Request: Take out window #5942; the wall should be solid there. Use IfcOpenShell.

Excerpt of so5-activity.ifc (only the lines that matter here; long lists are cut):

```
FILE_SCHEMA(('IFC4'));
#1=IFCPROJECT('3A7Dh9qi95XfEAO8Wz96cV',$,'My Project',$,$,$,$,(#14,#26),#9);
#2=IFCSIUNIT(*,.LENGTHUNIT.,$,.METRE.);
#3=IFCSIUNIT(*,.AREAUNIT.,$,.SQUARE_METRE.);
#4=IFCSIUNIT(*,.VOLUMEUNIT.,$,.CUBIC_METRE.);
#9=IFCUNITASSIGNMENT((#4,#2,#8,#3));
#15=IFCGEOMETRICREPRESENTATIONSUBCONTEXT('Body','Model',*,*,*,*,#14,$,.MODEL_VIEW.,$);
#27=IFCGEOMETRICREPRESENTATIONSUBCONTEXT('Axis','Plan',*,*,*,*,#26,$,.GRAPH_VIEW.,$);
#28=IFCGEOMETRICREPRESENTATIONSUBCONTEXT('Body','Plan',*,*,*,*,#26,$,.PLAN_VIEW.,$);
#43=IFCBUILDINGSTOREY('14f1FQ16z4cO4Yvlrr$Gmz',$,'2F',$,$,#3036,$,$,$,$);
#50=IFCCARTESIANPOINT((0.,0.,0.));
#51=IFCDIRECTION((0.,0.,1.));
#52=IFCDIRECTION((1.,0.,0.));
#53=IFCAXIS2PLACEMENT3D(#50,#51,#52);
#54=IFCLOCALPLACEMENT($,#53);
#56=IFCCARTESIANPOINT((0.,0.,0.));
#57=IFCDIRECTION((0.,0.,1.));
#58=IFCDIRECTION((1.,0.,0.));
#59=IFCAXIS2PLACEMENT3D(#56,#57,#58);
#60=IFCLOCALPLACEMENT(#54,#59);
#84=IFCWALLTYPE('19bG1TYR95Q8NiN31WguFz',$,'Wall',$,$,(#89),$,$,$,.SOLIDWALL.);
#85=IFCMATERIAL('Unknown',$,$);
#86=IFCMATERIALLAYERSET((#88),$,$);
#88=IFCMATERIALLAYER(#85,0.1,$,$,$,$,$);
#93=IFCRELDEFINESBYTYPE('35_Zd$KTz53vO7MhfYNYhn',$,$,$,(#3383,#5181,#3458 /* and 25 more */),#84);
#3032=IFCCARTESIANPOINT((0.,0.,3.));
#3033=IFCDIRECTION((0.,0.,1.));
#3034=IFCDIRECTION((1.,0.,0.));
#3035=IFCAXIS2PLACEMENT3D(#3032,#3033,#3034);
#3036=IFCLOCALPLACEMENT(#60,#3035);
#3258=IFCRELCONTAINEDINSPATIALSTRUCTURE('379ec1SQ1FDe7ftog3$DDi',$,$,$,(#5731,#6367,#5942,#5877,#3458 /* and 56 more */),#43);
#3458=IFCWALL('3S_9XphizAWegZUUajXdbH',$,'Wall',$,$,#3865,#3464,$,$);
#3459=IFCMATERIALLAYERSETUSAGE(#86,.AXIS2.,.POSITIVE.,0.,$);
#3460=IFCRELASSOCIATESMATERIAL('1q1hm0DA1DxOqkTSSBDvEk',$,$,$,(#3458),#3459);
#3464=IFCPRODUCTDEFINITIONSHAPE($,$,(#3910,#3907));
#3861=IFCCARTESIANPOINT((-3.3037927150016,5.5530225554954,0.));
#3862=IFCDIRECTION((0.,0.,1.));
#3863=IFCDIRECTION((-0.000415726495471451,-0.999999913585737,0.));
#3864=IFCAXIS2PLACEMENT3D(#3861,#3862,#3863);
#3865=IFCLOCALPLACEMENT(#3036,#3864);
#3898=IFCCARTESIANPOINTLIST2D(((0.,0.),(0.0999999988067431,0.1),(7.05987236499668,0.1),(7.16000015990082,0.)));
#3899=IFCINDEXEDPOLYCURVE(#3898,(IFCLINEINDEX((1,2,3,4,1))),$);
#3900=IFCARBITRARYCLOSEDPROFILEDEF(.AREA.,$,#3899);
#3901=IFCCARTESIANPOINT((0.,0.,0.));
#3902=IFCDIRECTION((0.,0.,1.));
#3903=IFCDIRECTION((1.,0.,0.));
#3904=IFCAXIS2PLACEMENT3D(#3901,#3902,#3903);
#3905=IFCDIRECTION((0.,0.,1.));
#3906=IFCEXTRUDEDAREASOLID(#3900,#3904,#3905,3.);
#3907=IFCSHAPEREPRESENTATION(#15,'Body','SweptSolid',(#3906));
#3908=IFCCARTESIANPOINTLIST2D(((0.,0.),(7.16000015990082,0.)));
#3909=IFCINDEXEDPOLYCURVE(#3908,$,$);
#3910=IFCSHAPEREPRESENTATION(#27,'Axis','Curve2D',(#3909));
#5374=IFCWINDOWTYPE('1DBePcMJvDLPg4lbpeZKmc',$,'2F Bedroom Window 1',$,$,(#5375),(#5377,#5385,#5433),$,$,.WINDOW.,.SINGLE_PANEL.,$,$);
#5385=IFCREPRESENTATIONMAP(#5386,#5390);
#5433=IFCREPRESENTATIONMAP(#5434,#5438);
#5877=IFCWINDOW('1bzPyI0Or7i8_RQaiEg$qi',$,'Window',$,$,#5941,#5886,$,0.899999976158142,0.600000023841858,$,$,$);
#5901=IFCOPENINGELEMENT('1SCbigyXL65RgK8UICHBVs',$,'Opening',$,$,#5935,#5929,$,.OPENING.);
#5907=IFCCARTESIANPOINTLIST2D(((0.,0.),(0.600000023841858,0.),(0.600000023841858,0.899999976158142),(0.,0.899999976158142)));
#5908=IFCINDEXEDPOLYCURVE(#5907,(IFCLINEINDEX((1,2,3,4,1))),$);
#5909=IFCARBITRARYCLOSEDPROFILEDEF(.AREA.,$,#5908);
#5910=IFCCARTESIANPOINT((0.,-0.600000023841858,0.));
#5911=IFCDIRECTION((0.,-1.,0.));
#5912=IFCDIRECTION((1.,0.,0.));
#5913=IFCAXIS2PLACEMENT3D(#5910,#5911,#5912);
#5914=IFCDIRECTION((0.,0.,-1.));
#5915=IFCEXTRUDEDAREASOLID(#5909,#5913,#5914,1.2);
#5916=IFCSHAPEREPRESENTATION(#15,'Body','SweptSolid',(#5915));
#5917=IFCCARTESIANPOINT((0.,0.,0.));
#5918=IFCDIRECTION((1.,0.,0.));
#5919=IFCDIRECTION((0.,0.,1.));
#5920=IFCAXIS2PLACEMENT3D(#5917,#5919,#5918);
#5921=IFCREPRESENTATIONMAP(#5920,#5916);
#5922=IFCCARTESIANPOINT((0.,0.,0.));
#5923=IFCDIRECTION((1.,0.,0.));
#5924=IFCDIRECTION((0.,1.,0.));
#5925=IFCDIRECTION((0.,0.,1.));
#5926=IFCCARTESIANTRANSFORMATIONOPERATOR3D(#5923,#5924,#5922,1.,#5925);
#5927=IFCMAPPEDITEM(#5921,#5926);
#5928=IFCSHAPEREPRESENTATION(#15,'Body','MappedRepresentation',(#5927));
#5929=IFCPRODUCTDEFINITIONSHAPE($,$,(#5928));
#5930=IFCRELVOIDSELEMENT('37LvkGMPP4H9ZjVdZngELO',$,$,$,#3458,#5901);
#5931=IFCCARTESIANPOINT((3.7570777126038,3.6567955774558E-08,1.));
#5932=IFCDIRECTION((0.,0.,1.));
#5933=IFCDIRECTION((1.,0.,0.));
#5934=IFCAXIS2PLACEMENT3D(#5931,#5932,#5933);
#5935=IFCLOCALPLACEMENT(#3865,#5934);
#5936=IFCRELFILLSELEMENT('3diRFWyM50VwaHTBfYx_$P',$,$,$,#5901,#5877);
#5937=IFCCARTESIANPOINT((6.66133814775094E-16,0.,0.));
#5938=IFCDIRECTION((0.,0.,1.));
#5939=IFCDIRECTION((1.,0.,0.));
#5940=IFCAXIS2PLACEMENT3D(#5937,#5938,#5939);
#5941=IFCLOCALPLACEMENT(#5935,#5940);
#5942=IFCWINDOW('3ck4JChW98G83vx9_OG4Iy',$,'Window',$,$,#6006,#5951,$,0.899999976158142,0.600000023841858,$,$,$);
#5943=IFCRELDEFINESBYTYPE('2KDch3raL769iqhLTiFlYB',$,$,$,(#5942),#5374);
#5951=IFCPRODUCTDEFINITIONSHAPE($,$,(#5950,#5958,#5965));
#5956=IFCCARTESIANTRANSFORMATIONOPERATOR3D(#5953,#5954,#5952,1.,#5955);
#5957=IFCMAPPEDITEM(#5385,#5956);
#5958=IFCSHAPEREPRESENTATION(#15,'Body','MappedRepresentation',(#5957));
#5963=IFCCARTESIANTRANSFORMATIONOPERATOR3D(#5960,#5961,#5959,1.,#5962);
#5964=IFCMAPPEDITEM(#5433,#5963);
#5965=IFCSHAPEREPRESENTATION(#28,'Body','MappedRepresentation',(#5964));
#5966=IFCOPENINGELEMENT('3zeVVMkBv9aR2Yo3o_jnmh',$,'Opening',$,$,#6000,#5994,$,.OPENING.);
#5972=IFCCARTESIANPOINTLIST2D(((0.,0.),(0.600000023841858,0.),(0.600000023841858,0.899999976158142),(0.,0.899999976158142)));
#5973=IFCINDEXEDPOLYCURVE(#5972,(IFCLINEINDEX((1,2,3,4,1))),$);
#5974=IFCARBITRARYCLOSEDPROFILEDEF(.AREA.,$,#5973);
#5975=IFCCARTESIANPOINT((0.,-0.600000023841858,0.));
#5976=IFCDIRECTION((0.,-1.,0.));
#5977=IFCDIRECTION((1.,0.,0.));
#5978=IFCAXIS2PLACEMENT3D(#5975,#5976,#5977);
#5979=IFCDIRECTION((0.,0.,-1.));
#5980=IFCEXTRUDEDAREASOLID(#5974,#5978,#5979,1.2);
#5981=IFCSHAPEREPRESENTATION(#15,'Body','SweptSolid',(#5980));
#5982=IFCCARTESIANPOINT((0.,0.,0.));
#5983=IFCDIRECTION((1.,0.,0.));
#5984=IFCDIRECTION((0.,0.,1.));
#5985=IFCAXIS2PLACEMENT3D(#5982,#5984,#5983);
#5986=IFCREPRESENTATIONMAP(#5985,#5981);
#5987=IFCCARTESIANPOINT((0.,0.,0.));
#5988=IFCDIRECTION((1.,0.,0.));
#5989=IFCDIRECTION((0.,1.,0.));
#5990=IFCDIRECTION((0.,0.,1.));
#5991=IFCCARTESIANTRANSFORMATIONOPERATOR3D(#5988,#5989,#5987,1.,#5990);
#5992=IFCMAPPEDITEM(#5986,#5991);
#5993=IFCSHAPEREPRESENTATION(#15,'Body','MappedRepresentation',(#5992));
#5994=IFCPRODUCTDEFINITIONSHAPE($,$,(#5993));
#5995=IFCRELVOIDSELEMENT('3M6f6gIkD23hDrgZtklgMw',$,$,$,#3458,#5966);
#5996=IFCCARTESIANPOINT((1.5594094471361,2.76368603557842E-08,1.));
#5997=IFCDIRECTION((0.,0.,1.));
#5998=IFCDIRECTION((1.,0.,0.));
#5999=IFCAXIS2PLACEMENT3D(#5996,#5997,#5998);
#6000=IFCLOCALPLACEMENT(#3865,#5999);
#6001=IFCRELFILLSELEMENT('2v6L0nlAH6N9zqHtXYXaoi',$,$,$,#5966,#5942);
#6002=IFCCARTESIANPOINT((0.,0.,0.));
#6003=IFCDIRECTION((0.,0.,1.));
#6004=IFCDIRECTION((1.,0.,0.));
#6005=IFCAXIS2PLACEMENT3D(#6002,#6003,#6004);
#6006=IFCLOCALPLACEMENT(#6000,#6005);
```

```python
import ifcopenshell
import ifcopenshell.api.feature
import ifcopenshell.api.root
import ifcopenshell.geom
import ifcopenshell.util.shape

model = ifcopenshell.open("so5-activity.ifc")
settings = ifcopenshell.geom.settings()


def volume(element):
    """Net volume in cubic metres, openings subtracted."""
    shape = ifcopenshell.geom.create_shape(settings, element)
    return ifcopenshell.util.shape.get_volume(shape.geometry)


window = model.by_id(5942)
opening = window.FillsVoids[0].RelatingOpeningElement
wall = opening.VoidsElements[0].RelatingBuildingElement
before = volume(wall)

ifcopenshell.api.root.remove_product(model, product=window)
ifcopenshell.api.feature.remove_feature(model, feature=opening)

after = volume(wall)

print(f"wall volume {before:.3f} -> {after:.3f} m3")

model.write("so5-activity_rev.ifc")
```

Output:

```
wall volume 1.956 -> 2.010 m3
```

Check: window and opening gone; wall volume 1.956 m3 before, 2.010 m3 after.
